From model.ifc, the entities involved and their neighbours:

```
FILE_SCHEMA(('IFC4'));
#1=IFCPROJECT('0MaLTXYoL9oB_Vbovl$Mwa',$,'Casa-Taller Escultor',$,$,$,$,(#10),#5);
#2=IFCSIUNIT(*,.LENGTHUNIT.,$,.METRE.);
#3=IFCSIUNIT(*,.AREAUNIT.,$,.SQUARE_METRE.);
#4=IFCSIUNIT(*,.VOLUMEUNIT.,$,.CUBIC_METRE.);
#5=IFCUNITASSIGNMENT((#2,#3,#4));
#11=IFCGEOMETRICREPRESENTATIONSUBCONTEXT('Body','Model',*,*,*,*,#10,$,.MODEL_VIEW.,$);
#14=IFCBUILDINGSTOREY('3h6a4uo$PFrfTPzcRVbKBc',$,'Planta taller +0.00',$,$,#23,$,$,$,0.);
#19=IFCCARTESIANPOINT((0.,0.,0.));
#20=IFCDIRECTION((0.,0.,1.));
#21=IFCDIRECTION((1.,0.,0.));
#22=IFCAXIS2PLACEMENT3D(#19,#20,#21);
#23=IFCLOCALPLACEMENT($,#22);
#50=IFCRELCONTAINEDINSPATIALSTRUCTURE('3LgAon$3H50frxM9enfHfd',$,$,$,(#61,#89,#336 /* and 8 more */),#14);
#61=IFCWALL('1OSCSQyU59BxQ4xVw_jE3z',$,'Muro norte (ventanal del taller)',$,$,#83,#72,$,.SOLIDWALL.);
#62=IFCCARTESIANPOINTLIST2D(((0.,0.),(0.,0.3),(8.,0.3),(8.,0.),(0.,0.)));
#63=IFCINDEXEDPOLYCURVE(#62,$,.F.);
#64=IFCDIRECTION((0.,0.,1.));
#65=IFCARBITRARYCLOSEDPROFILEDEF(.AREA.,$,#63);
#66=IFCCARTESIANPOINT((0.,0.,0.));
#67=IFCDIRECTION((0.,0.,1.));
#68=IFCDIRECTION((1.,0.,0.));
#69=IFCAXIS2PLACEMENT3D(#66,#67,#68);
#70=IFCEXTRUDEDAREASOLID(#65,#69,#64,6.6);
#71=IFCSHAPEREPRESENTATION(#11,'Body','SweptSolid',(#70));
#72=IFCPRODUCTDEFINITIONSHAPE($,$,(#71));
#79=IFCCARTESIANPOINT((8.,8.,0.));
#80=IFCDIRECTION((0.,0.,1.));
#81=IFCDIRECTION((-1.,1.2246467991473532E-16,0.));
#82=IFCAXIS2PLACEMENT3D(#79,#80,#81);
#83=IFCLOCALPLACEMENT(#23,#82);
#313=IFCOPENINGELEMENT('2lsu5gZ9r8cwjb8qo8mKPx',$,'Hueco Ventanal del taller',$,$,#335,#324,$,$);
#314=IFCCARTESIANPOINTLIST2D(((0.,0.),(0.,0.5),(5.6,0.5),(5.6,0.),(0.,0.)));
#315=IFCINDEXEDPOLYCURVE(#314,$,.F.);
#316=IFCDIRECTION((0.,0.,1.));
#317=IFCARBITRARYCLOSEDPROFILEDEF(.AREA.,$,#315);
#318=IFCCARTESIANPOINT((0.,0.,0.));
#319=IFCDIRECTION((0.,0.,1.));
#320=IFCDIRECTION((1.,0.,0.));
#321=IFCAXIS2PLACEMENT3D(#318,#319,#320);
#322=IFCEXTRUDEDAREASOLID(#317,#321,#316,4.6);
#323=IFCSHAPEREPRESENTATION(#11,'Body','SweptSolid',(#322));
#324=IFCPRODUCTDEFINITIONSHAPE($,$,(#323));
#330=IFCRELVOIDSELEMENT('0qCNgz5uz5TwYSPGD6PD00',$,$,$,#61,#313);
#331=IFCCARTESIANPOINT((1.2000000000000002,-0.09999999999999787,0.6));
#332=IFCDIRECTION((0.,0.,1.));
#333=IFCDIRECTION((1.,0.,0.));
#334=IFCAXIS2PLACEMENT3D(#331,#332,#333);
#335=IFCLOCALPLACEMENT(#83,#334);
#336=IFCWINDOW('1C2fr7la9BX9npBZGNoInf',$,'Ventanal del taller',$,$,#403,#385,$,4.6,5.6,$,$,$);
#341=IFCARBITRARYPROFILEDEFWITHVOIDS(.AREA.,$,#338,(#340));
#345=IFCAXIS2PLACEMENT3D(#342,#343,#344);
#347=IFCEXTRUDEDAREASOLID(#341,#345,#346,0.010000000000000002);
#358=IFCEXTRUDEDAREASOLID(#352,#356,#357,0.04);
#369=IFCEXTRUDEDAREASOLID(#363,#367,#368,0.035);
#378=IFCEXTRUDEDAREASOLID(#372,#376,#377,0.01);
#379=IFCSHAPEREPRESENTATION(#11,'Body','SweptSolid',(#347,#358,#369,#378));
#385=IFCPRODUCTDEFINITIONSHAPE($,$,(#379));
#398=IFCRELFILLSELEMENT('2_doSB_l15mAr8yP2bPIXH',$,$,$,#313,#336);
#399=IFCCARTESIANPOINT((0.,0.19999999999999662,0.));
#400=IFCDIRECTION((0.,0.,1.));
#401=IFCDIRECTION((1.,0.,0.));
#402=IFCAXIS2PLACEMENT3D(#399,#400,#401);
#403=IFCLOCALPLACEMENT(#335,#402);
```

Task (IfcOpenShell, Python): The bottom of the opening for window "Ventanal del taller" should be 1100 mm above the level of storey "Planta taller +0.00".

```python
import numpy as np
import ifcopenshell
import ifcopenshell.api.geometry
import ifcopenshell.geom
import ifcopenshell.util.element
import ifcopenshell.util.placement
import ifcopenshell.util.shape
import ifcopenshell.util.unit

model = ifcopenshell.open("model.ifc")
unit_scale = ifcopenshell.util.unit.calculate_unit_scale(model)

window = model.by_guid("1C2fr7la9BX9npBZGNoInf")
opening = window.FillsVoids[0].RelatingOpeningElement
storey = ifcopenshell.util.element.get_container(window, ifc_class="IfcBuildingStorey")
level = ifcopenshell.util.placement.get_local_placement(storey.ObjectPlacement)[2, 3]

# The opening's origin need not be at the sill, so measure its lowest point.
shape = ifcopenshell.geom.create_shape(ifcopenshell.geom.settings(), opening)
bottom = ifcopenshell.util.shape.get_shape_bottom_elevation(shape, shape.geometry) / unit_scale
dz = level + 1.1 / unit_scale - bottom

shift = np.array([0.0, 0.0, dz])
# The window is placed relative to its opening, so it follows when the opening moves.
matrix = ifcopenshell.util.placement.get_local_placement(opening.ObjectPlacement)
matrix[:3, 3] += shift
ifcopenshell.api.geometry.edit_object_placement(
    model, product=opening, matrix=matrix, is_si=False, should_transform_children=True
)

print(f"moved by {dz * unit_scale:+.3f} m")

model.write("model-out.ifc")
```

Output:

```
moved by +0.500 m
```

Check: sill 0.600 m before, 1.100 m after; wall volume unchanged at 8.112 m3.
